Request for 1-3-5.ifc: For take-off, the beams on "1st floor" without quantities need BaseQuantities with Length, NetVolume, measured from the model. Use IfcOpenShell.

First a look at what the model holds.

```python
import ifcopenshell
import ifcopenshell.util.element
import ifcopenshell.util.unit

model = ifcopenshell.open("1-3-5.ifc")
print(model.schema)
for unit_type in ("LENGTHUNIT", "AREAUNIT", "VOLUMEUNIT"):
    print(unit_type, ifcopenshell.util.unit.calculate_unit_scale(model, unit_type))
storey = next(s for s in model.by_type("IfcBuildingStorey") if s.Name == "1st floor")
beams = [e for e in ifcopenshell.util.element.get_decomposition(storey) if e.is_a("IfcBeam")]
for e in sorted(beams, key=lambda e: e.id()):
    print(e.id(), e.is_a(), e.Name, list(ifcopenshell.util.element.get_psets(e, qtos_only=True)), sep=" | ")
```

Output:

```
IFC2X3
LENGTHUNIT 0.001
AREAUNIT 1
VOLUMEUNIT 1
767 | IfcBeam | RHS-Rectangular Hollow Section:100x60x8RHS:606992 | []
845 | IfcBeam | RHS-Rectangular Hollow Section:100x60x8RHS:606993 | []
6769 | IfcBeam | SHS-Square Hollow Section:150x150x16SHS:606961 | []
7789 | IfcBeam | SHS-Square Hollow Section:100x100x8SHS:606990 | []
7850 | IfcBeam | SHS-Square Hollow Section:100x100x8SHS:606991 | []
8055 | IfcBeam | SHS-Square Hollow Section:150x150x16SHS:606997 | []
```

```python
import ifcopenshell
import ifcopenshell.api.pset
import ifcopenshell.geom
import ifcopenshell.util.element
import ifcopenshell.util.shape
import ifcopenshell.util.unit

model = ifcopenshell.open("1-3-5.ifc")
unit_scale = ifcopenshell.util.unit.calculate_unit_scale(model)
volume_scale = ifcopenshell.util.unit.calculate_unit_scale(model, "VOLUMEUNIT")
settings = ifcopenshell.geom.settings()

storey = next(s for s in model.by_type("IfcBuildingStorey") if s.Name == "1st floor")
beams = [e for e in ifcopenshell.util.element.get_decomposition(storey) if e.is_a("IfcBeam")]

for e in sorted(beams, key=lambda e: e.id()):
    if ifcopenshell.util.element.get_psets(e, qtos_only=True, should_inherit=False):
        continue
    # Geometry comes back in metres, in the element's own axes.
    shape = ifcopenshell.geom.create_shape(settings, e)
    values = {
        "Length": ifcopenshell.util.shape.get_max_xyz(shape.geometry) / unit_scale,
        "NetVolume": ifcopenshell.util.shape.get_volume(shape.geometry) / volume_scale,
    }
    qto = ifcopenshell.api.pset.add_qto(model, product=e, name="BaseQuantities")
    ifcopenshell.api.pset.edit_qto(model, qto=qto, properties=values)
    print(e.id(), {k: round(v, 3) for k, v in values.items()})

model.write("1-3-5_updated.ifc")
```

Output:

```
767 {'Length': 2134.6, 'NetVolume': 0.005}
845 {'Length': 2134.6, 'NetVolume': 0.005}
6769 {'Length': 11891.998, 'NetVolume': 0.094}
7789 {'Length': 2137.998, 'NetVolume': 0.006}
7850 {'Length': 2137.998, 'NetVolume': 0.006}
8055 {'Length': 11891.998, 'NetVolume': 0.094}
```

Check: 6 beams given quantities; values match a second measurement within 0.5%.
